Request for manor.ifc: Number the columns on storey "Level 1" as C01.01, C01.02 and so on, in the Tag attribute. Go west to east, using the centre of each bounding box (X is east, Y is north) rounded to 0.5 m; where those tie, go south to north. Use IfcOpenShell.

First a look at what the model holds.

```python
import ifcopenshell
import ifcopenshell.util.element
import ifcopenshell.util.placement

model = ifcopenshell.open("manor.ifc")
print(model.schema)
storey = next(s for s in model.by_type("IfcBuildingStorey") if s.Name == "Level 1")
columns = [e for e in ifcopenshell.util.element.get_decomposition(storey) if e.is_a("IfcColumn")]
for e in sorted(columns, key=lambda e: e.id()):
    origin = ifcopenshell.util.placement.get_local_placement(e.ObjectPlacement)[:3, 3]
    print(e.id(), e.Tag, e.Name, origin.round(2) + 0.0, sep=" | ")
```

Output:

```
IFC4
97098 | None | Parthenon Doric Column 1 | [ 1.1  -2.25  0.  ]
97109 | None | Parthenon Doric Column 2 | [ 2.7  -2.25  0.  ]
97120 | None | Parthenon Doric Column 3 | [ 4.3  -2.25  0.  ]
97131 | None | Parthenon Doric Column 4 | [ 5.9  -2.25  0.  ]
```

```python
import ifcopenshell
import ifcopenshell.geom
import ifcopenshell.util.element
import ifcopenshell.util.shape

model = ifcopenshell.open("manor.ifc")
settings = ifcopenshell.geom.settings()
settings.set("use-world-coords", True)


def centre(element):
    shape = ifcopenshell.geom.create_shape(settings, element)
    return ifcopenshell.util.shape.get_bbox_centroid(shape.geometry)


storey = next(s for s in model.by_type("IfcBuildingStorey") if s.Name == "Level 1")
columns = [e for e in ifcopenshell.util.element.get_decomposition(storey) if e.is_a("IfcColumn")]

# Insertion points can sit at a corner or the storey origin, so sort by the geometry (in metres).
centres = {e: centre(e) for e in columns}
columns.sort(key=lambda e: (round(centres[e][0] / 0.5), centres[e][1]))

for i, e in enumerate(columns, start=1):
    number = f"C01.{i:02d}"
    e.Tag = number
    print(e.id(), number)

model.write("manor-out.ifc")
```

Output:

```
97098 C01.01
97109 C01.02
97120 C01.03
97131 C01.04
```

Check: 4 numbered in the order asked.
